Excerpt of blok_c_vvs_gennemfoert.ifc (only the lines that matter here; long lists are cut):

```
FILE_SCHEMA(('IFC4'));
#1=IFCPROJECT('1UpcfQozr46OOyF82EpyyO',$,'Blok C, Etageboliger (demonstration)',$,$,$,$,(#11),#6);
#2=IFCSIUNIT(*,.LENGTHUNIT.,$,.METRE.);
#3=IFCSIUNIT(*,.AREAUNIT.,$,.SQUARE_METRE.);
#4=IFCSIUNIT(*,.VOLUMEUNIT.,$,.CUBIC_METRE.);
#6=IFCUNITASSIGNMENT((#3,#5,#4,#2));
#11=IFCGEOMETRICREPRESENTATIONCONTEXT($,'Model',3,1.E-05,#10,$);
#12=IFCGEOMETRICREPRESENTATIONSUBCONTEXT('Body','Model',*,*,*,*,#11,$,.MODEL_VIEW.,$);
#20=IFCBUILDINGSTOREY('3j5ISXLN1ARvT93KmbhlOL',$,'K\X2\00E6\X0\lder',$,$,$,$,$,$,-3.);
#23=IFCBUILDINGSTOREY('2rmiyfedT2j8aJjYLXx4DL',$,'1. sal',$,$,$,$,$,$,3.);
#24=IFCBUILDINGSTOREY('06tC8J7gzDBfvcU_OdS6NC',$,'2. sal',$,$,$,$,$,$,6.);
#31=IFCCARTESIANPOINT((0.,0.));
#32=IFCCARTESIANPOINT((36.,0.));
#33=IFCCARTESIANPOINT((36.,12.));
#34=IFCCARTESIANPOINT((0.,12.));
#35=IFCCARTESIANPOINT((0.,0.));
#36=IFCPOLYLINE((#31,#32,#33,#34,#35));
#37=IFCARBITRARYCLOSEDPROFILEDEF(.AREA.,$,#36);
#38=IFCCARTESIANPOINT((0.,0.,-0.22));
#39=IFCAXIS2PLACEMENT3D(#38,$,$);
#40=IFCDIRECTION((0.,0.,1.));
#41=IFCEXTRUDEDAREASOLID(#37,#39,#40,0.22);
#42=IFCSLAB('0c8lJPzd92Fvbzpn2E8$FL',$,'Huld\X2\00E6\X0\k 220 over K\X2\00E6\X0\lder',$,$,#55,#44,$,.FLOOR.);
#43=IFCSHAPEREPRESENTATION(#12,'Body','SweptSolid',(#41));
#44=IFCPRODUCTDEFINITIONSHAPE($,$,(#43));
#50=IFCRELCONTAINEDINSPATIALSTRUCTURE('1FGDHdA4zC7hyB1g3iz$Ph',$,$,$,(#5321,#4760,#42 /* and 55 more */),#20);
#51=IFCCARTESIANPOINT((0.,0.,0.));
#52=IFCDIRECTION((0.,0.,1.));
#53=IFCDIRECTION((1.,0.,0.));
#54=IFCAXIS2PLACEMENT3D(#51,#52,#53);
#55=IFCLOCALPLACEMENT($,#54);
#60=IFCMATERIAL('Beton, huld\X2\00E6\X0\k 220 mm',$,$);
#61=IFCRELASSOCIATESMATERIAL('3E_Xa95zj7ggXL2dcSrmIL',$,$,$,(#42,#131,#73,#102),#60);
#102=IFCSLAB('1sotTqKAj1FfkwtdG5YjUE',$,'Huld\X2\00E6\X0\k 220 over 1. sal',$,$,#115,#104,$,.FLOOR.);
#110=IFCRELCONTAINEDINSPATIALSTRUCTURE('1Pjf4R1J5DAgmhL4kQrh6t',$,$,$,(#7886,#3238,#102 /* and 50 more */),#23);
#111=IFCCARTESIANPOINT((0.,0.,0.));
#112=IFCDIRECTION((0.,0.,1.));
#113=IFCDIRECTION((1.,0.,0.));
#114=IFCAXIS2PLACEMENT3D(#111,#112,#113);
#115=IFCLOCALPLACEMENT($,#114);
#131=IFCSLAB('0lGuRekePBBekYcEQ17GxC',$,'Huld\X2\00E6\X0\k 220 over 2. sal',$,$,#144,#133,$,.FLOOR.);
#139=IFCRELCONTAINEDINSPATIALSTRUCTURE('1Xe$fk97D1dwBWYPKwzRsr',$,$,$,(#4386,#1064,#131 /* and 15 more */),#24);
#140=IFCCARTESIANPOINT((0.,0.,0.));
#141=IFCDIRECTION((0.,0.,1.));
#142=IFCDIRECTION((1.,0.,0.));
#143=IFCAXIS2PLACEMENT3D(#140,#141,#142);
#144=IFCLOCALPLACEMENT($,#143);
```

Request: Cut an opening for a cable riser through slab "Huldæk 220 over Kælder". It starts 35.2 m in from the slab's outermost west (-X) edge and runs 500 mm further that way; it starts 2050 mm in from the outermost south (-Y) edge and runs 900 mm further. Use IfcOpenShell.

```python
import numpy as np
import ifcopenshell
import ifcopenshell.api.feature
import ifcopenshell.api.geometry
import ifcopenshell.api.root
import ifcopenshell.geom
import ifcopenshell.util.placement
import ifcopenshell.util.representation
import ifcopenshell.util.shape
import ifcopenshell.util.unit

model = ifcopenshell.open("blok_c_vvs_gennemfoert.ifc")
unit_scale = ifcopenshell.util.unit.calculate_unit_scale(model)
settings = ifcopenshell.geom.settings()


def volume(element):
    """Net volume in cubic metres, openings subtracted."""
    shape = ifcopenshell.geom.create_shape(settings, element)
    return ifcopenshell.util.shape.get_volume(shape.geometry)


slab = model.by_id(42)
before = volume(slab)

# Extent in the slab's own axes, in metres. The edges named are its -X and -Y sides.
slab_shape = ifcopenshell.geom.create_shape(settings, slab)
vertices = ifcopenshell.util.shape.get_vertices(slab_shape.geometry)
x_min, y_min, bottom = vertices.min(axis=0)
top = vertices[:, 2].max()

opening = ifcopenshell.api.root.create_entity(model, ifc_class="IfcOpeningElement", name="Cable riser opening", predefined_type="OPENING")
context = ifcopenshell.util.representation.get_context(model, "Model", "Body", "MODEL_VIEW")
width, depth = 0.5, 0.9
outline = [(0.0, 0.0), (width, 0.0), (width, depth), (0.0, depth), (0.0, 0.0)]
# Overshoot both faces by 50 mm so the cut is clean.
shape = ifcopenshell.api.geometry.add_slab_representation(
    model, context=context, depth=top - bottom + 0.1, polyline=outline
)
ifcopenshell.api.geometry.assign_representation(model, product=opening, representation=shape)

matrix = ifcopenshell.util.placement.get_local_placement(slab.ObjectPlacement)
matrix[:, 3] = matrix @ np.append(np.array([x_min + 35.2, y_min + 2.05, bottom - 0.05]) / unit_scale, 1.0)
ifcopenshell.api.geometry.edit_object_placement(model, product=opening, matrix=matrix, is_si=False)
ifcopenshell.api.feature.add_feature(model, feature=opening, element=slab)

after = volume(slab)

print(f"slab volume {before:.3f} -> {after:.3f} m3")

model.write("blok_c_vvs_gennemfoert-out.ifc")
```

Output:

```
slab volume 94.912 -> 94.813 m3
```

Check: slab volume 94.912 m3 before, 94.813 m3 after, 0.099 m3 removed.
